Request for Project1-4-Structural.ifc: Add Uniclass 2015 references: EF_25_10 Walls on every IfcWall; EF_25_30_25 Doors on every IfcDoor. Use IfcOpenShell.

First a look at what the model holds.

```python
import ifcopenshell

model = ifcopenshell.open("Project1-4-Structural.ifc")
print(model.schema)
print("classifications:", [c.Name for c in model.by_type("IfcClassification")])
for ifc_class in ("IfcDoor", "IfcRoof", "IfcStair", "IfcWall", "IfcWindow"):
    print(ifc_class, len(model.by_type(ifc_class)))
```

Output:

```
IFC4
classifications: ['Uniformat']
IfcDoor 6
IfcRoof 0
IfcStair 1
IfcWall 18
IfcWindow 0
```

```python
import ifcopenshell
import ifcopenshell.api.classification

model = ifcopenshell.open("Project1-4-Structural.ifc")

system = ifcopenshell.api.classification.add_classification(model, classification="Uniclass 2015")

codes = {
    "IfcWall": ("EF_25_10", "Walls"),
    "IfcDoor": ("EF_25_30_25", "Doors"),
}
for ifc_class, (code, name) in codes.items():
    products = model.by_type(ifc_class)
    ifcopenshell.api.classification.add_reference(
        model, products=products, classification=system, identification=code, name=name
    )
    print(code, len(products))

model.write("Project1-4-Structural_edited.ifc")
```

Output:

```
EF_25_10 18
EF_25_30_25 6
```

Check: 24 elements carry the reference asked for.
